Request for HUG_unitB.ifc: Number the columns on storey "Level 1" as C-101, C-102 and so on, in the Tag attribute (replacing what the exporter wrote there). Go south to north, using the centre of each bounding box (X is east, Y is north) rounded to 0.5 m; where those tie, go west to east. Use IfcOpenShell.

First a look at what the model holds.

```python
import ifcopenshell
import ifcopenshell.util.element
import ifcopenshell.util.placement

model = ifcopenshell.open("HUG_unitB.ifc")
print(model.schema)
storey = next(s for s in model.by_type("IfcBuildingStorey") if s.Name == "Level 1")
columns = [e for e in ifcopenshell.util.element.get_decomposition(storey) if e.is_a("IfcColumn")]
for e in sorted(columns, key=lambda e: e.id()):
    origin = ifcopenshell.util.placement.get_local_placement(e.ObjectPlacement)[:3, 3]
    print(e.id(), e.Tag, e.Name, origin.round(2) + 0.0, sep=" | ")
```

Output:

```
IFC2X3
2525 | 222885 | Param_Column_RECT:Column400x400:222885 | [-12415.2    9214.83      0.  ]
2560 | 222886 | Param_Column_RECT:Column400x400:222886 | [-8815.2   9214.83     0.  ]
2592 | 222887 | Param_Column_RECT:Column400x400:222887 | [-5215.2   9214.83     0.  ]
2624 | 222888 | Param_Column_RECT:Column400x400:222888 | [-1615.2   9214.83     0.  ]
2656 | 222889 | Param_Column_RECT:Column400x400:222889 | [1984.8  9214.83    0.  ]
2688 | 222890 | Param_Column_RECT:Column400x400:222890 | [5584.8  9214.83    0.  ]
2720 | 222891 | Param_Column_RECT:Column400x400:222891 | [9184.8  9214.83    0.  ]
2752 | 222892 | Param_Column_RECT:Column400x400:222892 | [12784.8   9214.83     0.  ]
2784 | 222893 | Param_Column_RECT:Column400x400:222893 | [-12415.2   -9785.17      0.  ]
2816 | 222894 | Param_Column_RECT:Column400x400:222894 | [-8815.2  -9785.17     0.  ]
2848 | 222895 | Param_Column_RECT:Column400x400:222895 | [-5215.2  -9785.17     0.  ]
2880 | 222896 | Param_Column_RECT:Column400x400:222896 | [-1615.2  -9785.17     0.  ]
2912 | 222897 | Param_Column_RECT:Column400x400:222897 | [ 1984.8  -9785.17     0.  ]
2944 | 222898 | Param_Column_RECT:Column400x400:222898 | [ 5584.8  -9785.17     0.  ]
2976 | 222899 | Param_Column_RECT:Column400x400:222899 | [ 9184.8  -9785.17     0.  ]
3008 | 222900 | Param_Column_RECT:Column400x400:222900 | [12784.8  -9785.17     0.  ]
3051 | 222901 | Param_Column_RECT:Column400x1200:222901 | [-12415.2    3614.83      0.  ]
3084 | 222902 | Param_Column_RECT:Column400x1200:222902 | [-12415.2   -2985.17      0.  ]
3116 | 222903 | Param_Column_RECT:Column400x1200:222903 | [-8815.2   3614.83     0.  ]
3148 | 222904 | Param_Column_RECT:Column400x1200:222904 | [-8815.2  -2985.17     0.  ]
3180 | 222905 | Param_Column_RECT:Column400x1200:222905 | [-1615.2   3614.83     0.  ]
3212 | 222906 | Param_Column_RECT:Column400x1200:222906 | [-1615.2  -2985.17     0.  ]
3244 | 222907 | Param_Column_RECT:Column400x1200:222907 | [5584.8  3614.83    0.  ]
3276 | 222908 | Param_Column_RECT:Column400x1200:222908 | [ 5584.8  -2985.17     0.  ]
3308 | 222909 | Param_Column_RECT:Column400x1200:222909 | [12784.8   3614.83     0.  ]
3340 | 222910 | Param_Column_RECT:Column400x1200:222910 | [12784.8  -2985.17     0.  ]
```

```python
import ifcopenshell
import ifcopenshell.geom
import ifcopenshell.util.element
import ifcopenshell.util.shape

model = ifcopenshell.open("HUG_unitB.ifc")
settings = ifcopenshell.geom.settings()
settings.set("use-world-coords", True)


def centre(element):
    shape = ifcopenshell.geom.create_shape(settings, element)
    return ifcopenshell.util.shape.get_bbox_centroid(shape.geometry)


storey = next(s for s in model.by_type("IfcBuildingStorey") if s.Name == "Level 1")
columns = [e for e in ifcopenshell.util.element.get_decomposition(storey) if e.is_a("IfcColumn")]

# Insertion points can sit at a corner or the storey origin, so sort by the geometry (in metres).
centres = {e: centre(e) for e in columns}
columns.sort(key=lambda e: (round(centres[e][1] / 0.5), centres[e][0]))

for i, e in enumerate(columns, start=1):
    number = f"C-1{i:02d}"
    e.Tag = number
    print(e.id(), number)

model.write("HUG_unitB_rev.ifc")
```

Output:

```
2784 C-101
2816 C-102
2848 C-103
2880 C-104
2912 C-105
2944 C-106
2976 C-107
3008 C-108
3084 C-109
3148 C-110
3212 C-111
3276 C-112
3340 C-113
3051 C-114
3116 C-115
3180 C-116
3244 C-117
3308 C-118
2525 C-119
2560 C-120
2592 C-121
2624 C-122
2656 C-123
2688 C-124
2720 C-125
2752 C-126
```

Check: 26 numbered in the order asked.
